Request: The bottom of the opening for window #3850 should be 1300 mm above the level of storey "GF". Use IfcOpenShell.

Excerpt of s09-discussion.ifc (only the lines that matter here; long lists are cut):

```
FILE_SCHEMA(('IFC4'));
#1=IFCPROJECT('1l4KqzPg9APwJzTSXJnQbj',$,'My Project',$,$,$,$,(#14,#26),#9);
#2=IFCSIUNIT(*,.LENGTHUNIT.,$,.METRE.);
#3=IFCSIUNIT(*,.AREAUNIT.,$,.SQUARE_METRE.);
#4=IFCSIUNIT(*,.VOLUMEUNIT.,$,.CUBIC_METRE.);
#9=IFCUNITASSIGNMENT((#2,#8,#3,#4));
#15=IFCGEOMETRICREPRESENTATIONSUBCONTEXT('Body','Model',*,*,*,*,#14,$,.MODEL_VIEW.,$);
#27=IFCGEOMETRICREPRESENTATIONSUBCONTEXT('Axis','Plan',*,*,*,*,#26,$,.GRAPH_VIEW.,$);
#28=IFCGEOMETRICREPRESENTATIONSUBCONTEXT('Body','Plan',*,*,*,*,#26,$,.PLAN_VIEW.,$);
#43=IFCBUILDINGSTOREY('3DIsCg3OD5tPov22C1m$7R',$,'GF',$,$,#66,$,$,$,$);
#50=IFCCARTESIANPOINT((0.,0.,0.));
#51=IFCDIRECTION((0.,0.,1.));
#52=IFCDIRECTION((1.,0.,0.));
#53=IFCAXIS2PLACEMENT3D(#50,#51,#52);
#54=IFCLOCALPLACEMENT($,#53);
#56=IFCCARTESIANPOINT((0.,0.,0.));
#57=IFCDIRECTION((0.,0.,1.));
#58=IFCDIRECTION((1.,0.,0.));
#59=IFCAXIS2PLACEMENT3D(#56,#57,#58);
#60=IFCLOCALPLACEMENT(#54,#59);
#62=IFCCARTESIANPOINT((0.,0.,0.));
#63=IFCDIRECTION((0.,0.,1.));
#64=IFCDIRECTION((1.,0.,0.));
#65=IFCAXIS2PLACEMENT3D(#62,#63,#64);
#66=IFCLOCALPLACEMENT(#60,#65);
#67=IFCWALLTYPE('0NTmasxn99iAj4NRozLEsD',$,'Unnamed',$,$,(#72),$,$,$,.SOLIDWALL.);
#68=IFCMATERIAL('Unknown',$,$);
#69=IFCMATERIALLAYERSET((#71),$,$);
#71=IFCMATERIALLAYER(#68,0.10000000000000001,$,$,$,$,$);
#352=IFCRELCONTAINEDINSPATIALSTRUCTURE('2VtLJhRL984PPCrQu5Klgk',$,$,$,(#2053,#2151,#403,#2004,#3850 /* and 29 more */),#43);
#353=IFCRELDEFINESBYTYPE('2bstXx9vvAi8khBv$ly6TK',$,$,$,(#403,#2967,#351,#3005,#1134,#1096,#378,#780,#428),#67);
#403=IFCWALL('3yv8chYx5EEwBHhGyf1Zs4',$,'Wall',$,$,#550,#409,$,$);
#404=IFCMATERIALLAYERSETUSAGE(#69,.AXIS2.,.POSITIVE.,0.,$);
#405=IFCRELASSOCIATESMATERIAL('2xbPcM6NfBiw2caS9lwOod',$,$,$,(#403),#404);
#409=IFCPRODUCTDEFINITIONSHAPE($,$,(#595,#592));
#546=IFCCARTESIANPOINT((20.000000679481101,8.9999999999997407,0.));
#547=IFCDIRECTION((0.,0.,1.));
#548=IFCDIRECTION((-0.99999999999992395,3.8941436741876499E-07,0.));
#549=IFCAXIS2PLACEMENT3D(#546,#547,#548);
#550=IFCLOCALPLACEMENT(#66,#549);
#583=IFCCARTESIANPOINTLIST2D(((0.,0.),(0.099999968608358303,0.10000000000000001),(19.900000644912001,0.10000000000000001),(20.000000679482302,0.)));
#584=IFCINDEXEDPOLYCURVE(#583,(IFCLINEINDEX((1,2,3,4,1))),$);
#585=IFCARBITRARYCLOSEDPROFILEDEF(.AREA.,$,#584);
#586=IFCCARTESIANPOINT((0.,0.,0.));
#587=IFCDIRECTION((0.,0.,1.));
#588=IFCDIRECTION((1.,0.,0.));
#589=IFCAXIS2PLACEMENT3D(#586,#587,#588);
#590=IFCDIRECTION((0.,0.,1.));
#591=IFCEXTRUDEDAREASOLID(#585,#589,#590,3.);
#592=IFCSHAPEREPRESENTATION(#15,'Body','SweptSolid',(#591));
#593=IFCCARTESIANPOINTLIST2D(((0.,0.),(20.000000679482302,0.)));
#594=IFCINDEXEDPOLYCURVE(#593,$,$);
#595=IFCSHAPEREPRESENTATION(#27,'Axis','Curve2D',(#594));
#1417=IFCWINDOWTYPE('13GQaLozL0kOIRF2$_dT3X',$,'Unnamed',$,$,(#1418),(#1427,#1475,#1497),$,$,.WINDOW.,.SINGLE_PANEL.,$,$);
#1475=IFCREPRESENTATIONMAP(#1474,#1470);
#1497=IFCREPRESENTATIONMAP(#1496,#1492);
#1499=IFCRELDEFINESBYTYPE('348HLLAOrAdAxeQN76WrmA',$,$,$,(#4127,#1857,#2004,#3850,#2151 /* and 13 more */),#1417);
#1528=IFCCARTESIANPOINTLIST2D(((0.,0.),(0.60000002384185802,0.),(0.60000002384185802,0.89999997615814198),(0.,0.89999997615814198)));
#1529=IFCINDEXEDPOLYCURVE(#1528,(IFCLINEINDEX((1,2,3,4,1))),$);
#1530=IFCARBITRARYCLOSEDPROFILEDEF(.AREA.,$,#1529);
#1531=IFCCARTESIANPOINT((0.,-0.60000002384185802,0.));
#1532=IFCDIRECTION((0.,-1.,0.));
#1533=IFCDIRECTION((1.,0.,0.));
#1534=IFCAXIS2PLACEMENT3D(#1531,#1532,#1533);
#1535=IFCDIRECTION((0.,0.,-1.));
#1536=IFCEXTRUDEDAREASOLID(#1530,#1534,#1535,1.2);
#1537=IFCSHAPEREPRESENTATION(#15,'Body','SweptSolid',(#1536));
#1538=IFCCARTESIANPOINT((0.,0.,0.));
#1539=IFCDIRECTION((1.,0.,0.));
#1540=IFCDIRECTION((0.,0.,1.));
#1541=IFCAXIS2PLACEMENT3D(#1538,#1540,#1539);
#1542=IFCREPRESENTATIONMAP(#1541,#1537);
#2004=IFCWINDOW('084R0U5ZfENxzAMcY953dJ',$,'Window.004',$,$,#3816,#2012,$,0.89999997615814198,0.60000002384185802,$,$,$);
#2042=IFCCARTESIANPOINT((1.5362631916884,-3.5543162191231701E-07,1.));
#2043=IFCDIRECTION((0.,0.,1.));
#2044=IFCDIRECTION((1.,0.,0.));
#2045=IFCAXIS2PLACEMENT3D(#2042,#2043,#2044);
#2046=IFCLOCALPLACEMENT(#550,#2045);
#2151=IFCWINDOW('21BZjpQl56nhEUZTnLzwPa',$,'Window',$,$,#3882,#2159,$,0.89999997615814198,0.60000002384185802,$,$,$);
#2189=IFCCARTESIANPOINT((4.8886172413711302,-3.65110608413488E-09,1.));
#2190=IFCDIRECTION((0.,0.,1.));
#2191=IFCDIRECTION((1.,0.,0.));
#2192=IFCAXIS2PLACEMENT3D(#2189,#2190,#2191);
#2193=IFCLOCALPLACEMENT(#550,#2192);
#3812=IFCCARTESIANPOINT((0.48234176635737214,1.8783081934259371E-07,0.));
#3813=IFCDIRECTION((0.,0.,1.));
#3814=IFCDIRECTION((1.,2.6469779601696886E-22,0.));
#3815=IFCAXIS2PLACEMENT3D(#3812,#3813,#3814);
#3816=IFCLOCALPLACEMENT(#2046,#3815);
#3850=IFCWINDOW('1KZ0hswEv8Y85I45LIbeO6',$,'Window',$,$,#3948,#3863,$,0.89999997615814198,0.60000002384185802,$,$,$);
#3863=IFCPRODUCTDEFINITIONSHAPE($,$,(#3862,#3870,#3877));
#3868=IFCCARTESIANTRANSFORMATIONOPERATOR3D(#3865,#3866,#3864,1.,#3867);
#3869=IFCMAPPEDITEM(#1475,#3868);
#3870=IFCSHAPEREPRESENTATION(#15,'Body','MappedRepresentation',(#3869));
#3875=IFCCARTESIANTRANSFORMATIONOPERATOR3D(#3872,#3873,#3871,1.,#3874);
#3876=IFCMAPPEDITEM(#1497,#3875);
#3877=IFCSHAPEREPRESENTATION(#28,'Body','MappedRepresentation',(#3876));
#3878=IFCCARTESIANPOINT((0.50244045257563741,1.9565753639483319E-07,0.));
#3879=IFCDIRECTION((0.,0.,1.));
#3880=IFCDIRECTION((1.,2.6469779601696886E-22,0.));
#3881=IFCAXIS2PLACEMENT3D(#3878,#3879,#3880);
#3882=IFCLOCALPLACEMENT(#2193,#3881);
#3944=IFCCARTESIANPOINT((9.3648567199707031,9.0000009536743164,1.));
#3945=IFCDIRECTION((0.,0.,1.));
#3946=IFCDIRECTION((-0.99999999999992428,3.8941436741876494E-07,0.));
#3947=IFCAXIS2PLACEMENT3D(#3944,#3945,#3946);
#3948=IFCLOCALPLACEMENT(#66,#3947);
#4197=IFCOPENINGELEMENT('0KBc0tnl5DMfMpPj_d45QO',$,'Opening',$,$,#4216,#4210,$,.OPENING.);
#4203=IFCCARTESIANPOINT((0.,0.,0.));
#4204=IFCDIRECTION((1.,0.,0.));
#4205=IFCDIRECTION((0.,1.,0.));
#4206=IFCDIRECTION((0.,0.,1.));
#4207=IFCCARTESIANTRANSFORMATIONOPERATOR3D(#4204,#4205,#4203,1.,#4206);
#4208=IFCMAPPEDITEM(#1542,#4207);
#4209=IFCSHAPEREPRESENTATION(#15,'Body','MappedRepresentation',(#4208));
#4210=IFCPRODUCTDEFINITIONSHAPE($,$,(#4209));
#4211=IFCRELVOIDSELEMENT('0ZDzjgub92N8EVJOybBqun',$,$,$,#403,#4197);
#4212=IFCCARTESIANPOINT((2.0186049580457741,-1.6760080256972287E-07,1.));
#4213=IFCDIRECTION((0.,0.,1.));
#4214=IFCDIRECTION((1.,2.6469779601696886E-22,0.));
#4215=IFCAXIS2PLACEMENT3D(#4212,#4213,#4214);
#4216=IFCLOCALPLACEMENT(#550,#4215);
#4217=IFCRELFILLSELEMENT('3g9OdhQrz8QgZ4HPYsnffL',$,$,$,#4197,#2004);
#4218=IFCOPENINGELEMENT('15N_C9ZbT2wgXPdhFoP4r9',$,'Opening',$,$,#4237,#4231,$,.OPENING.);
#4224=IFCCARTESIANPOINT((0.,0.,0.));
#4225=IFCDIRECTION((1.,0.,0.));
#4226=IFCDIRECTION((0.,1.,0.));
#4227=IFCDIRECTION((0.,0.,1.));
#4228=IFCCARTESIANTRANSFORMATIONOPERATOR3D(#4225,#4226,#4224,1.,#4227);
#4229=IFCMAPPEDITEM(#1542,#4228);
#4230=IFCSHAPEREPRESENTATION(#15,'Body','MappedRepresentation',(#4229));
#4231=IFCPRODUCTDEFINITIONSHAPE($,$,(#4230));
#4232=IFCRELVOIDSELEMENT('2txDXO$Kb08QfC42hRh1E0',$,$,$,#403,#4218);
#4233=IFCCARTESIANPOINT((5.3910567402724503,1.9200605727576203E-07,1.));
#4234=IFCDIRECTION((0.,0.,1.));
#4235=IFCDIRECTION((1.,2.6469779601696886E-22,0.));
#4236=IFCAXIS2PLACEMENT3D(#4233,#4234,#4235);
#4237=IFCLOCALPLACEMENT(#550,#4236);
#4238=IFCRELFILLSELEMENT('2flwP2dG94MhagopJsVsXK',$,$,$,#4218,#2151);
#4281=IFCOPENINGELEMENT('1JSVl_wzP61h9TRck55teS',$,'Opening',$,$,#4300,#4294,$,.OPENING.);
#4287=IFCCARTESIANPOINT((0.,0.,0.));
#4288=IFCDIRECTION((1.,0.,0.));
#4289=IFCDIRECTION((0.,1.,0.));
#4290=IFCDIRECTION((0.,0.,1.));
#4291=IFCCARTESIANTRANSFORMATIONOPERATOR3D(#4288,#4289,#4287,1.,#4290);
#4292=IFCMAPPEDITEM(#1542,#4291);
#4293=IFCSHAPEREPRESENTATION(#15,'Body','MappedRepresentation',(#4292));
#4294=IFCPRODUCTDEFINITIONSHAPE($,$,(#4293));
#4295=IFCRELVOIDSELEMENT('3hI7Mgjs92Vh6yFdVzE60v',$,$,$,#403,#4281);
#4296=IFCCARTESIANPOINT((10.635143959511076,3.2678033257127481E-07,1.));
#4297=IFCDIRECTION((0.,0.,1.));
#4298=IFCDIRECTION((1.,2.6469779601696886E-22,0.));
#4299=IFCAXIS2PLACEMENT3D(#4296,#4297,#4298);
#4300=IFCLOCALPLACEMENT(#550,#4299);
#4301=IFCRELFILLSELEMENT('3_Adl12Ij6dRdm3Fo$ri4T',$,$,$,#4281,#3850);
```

```python
import numpy as np
import ifcopenshell
import ifcopenshell.api.geometry
import ifcopenshell.geom
import ifcopenshell.util.element
import ifcopenshell.util.placement
import ifcopenshell.util.shape
import ifcopenshell.util.unit

model = ifcopenshell.open("s09-discussion.ifc")
unit_scale = ifcopenshell.util.unit.calculate_unit_scale(model)

window = model.by_guid("1KZ0hswEv8Y85I45LIbeO6")
opening = window.FillsVoids[0].RelatingOpeningElement
storey = ifcopenshell.util.element.get_container(window, ifc_class="IfcBuildingStorey")
level = ifcopenshell.util.placement.get_local_placement(storey.ObjectPlacement)[2, 3]

# The opening's origin need not be at the sill, so measure its lowest point.
shape = ifcopenshell.geom.create_shape(ifcopenshell.geom.settings(), opening)
bottom = ifcopenshell.util.shape.get_shape_bottom_elevation(shape, shape.geometry) / unit_scale
dz = level + 1.3 / unit_scale - bottom

shift = np.array([0.0, 0.0, dz])
# The window is not placed relative to its opening, so move both.
for product in (opening, window):
    matrix = ifcopenshell.util.placement.get_local_placement(product.ObjectPlacement)
    matrix[:3, 3] += shift
    ifcopenshell.api.geometry.edit_object_placement(model, product=product, matrix=matrix, is_si=False)

print(f"moved by {dz * unit_scale:+.3f} m")

model.write("s09-discussion-out.ifc")
```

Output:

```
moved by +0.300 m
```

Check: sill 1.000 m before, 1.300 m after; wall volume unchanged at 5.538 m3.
